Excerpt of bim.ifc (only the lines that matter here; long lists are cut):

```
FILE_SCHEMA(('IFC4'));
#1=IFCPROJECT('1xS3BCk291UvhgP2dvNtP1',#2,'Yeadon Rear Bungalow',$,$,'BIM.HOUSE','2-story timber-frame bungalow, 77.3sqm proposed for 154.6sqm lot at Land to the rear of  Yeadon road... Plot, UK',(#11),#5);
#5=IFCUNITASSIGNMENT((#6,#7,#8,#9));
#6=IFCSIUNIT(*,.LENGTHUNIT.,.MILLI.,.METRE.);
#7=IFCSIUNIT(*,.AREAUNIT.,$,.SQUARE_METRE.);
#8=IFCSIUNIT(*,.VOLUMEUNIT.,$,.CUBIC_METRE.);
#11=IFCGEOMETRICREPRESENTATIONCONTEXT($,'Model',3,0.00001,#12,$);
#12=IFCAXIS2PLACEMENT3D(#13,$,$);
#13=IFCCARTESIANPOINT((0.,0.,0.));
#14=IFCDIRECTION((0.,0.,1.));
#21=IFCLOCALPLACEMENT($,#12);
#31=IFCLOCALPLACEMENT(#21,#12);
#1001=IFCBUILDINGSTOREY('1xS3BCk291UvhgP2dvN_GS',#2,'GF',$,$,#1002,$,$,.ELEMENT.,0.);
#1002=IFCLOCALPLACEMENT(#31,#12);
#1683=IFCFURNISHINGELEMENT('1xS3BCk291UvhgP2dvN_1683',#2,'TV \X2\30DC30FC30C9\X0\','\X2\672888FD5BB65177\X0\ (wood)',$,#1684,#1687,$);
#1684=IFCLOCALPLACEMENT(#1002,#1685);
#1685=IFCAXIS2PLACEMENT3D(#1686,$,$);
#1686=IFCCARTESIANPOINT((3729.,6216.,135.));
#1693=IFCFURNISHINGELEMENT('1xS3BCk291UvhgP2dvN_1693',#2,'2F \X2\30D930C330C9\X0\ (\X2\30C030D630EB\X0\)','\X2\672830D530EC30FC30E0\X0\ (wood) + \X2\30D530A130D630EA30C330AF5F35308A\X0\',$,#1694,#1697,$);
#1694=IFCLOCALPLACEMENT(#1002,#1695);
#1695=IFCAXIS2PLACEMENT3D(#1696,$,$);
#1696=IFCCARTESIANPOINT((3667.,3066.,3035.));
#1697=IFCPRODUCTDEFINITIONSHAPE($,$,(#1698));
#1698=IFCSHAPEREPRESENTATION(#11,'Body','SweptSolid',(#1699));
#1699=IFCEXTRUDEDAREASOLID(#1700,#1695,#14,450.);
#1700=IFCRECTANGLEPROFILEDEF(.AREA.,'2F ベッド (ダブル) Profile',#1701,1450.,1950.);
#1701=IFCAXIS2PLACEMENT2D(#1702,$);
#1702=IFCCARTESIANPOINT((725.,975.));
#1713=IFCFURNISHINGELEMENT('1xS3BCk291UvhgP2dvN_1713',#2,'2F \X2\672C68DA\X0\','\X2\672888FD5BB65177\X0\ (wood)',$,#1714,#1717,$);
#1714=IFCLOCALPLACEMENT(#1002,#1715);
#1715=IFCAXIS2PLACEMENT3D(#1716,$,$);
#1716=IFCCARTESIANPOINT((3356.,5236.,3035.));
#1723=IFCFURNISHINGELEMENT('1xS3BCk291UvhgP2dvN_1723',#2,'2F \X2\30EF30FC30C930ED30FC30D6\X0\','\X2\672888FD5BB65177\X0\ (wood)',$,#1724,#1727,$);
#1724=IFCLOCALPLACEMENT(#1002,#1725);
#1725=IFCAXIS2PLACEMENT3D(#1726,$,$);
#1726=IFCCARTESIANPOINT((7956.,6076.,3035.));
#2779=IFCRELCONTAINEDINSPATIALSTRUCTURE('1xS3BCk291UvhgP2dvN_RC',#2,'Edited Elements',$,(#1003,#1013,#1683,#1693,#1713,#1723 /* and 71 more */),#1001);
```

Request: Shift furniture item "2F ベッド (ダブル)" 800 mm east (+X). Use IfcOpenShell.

```python
import ifcopenshell
import ifcopenshell.api.geometry
import ifcopenshell.util.placement
import ifcopenshell.util.unit

model = ifcopenshell.open("bim.ifc")
unit_scale = ifcopenshell.util.unit.calculate_unit_scale(model)

item = model.by_id(1693)
matrix = ifcopenshell.util.placement.get_local_placement(item.ObjectPlacement)
matrix[0, 3] += 0.8 / unit_scale
ifcopenshell.api.geometry.edit_object_placement(model, product=item, matrix=matrix, is_si=False)

print(ifcopenshell.util.placement.get_local_placement(item.ObjectPlacement).round(3) + 0.0)

model.write("bim_rev.ifc")
```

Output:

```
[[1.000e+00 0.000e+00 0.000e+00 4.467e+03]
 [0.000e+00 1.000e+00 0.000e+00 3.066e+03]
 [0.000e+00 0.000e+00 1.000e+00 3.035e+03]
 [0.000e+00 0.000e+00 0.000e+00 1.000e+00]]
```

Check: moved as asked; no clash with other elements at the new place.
